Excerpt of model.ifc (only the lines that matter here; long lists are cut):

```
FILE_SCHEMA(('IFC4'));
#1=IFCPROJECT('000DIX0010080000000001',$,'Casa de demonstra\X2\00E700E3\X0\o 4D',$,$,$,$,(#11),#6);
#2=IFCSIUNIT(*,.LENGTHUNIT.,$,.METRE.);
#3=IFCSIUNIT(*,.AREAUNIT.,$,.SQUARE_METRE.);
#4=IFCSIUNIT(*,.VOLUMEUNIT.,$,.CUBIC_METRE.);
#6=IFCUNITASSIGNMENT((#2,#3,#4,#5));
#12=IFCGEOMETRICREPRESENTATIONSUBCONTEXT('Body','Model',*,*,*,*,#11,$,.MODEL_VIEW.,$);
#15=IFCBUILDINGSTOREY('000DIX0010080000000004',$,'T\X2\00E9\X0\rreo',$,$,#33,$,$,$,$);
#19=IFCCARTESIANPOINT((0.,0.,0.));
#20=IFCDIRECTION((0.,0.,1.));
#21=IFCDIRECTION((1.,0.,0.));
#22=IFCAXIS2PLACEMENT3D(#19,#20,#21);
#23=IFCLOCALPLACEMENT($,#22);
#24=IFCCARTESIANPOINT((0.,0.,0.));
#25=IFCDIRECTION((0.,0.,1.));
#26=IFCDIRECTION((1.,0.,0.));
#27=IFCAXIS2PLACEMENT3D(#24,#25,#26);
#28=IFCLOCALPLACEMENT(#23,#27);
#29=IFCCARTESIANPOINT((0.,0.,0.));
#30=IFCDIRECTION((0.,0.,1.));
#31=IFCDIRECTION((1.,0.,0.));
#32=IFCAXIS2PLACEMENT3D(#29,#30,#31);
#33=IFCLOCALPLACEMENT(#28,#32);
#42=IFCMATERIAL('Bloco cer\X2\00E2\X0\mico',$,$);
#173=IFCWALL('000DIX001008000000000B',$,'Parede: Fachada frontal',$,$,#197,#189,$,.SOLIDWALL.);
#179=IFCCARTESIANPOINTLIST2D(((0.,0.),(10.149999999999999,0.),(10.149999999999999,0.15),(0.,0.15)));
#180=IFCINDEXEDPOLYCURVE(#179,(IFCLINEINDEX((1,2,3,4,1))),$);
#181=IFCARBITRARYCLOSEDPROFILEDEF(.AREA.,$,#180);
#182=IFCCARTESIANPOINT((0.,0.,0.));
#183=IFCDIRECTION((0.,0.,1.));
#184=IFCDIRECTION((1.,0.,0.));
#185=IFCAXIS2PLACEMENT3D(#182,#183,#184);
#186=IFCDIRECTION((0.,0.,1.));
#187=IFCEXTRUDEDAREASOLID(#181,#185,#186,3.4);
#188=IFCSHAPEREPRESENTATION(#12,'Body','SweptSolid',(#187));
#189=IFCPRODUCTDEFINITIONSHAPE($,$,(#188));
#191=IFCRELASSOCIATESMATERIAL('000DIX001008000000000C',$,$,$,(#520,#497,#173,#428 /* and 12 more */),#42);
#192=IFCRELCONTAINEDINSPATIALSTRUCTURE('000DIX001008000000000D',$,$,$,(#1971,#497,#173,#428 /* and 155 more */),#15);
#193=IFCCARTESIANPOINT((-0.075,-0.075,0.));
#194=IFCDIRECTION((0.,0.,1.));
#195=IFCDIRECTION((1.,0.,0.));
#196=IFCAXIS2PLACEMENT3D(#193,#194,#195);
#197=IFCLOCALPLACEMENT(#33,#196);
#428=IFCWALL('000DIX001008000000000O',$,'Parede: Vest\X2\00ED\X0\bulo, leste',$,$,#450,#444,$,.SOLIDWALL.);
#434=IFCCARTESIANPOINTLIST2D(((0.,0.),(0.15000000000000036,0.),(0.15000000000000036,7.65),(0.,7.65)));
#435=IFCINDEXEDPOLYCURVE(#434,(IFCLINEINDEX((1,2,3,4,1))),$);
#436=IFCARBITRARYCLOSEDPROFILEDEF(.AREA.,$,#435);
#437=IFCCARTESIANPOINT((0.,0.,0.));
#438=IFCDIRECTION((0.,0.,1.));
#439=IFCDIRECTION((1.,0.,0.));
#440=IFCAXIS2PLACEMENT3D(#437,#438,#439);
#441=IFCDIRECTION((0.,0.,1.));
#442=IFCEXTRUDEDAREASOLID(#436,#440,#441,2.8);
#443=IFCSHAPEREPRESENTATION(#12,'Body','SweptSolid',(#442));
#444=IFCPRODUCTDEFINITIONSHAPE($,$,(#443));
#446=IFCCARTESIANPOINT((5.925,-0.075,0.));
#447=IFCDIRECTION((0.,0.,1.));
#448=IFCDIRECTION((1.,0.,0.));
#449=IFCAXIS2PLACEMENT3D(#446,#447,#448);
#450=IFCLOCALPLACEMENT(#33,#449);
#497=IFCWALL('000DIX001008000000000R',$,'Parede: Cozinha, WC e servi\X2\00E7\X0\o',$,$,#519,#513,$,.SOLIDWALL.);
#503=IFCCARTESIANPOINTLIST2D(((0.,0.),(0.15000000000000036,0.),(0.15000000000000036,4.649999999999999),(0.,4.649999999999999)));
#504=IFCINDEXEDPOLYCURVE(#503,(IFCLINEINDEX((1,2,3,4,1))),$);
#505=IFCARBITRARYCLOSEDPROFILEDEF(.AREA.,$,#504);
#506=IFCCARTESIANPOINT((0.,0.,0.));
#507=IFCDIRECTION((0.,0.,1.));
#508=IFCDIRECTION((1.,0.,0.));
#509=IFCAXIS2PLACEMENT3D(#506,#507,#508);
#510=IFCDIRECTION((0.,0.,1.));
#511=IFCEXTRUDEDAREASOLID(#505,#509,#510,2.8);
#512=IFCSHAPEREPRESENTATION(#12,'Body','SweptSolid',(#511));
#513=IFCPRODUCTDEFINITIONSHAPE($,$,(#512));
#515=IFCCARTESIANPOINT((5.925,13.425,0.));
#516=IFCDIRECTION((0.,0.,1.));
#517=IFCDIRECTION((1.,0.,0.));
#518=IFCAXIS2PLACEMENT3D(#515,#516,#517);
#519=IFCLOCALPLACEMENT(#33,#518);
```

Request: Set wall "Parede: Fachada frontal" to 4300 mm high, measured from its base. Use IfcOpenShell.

```python
import ifcopenshell
import ifcopenshell.geom
import ifcopenshell.util.representation
import ifcopenshell.util.shape
import ifcopenshell.util.unit

model = ifcopenshell.open("model.ifc")
unit_scale = ifcopenshell.util.unit.calculate_unit_scale(model)
settings = ifcopenshell.geom.settings()


def volume(element):
    """Net volume in cubic metres, openings subtracted."""
    shape = ifcopenshell.geom.create_shape(settings, element)
    return ifcopenshell.util.shape.get_volume(shape.geometry)


wall = model.by_guid("000DIX001008000000000B")
before = volume(wall)

body = ifcopenshell.util.representation.get_representation(wall, "Model", "Body")
solid = body.Items[0]
old_height = solid.Depth
solid.Depth = 4.3 / unit_scale
after = volume(wall)

print(f"height {old_height:g} -> {solid.Depth:g}, volume {before:.3f} -> {after:.3f} m3")

model.write("model_v2.ifc")
```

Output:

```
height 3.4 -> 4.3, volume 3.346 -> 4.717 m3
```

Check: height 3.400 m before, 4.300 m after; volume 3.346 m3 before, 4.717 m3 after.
